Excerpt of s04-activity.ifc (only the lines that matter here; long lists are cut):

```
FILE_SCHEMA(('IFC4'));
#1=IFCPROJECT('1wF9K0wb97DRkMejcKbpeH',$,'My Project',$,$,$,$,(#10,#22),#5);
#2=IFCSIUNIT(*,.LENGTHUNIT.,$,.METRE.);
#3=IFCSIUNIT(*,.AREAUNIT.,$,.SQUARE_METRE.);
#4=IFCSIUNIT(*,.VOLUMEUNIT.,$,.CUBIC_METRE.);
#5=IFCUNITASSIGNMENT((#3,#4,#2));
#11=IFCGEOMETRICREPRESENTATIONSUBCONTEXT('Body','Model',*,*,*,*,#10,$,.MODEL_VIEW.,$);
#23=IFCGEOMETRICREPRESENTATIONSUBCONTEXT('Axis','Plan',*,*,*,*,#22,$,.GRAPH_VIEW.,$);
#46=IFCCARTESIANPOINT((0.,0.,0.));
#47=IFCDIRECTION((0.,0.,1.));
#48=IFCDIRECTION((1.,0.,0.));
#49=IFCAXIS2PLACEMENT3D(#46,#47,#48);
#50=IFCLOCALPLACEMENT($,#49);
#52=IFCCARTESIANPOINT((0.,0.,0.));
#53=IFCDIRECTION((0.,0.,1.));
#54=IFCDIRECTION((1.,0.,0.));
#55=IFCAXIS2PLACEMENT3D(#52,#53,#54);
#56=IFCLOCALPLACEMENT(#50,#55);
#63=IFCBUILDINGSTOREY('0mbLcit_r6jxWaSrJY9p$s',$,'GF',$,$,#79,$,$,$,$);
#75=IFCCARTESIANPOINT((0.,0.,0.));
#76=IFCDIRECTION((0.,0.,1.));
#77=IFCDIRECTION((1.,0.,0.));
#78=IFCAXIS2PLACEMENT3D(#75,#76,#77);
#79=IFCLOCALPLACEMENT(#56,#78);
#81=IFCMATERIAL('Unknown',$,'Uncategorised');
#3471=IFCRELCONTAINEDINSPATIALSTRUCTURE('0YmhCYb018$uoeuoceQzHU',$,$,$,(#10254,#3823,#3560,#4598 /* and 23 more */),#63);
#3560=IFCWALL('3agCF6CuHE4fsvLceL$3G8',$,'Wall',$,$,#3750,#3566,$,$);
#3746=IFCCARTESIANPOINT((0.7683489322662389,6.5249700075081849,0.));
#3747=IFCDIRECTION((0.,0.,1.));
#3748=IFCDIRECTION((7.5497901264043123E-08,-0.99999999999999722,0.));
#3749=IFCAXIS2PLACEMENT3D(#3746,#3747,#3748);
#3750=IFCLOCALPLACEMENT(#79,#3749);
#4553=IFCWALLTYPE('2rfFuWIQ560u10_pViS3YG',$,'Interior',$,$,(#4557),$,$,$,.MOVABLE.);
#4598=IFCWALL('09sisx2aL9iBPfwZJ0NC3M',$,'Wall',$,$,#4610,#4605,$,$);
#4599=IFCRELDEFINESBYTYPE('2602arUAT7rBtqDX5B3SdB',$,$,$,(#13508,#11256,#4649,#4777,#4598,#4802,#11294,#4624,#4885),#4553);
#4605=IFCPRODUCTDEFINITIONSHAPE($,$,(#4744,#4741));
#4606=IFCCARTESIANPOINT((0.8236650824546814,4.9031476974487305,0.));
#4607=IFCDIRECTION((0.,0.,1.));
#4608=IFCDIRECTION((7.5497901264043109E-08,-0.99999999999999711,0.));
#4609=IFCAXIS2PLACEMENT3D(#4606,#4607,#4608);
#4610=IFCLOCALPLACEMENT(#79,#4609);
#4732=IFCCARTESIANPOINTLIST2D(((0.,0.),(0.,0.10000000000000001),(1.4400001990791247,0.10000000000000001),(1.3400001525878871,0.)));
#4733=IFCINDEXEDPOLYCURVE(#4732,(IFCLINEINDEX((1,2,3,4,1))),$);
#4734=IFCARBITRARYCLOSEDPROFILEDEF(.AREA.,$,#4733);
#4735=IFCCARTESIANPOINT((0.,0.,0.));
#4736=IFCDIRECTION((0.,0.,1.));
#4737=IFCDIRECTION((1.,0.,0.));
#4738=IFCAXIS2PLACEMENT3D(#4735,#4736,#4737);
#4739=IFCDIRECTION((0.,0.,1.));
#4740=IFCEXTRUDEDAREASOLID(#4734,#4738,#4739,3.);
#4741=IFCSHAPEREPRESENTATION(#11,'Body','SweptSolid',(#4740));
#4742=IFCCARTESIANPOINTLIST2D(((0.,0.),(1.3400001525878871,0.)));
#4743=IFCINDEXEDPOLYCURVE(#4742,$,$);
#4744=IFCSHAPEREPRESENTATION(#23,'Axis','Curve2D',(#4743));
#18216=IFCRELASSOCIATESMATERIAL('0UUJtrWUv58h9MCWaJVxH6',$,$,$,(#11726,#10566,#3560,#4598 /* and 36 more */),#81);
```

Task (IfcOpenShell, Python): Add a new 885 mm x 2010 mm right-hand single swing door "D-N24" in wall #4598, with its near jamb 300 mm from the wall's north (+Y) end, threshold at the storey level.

```python
import numpy as np
import ifcopenshell
import ifcopenshell.api.feature
import ifcopenshell.api.geometry
import ifcopenshell.api.root
import ifcopenshell.api.spatial
import ifcopenshell.geom
import ifcopenshell.util.element
import ifcopenshell.util.placement
import ifcopenshell.util.representation
import ifcopenshell.util.shape
import ifcopenshell.util.unit

model = ifcopenshell.open("s04-activity.ifc")
unit_scale = ifcopenshell.util.unit.calculate_unit_scale(model)
settings = ifcopenshell.geom.settings()


def volume(element):
    """Net volume in cubic metres, openings subtracted."""
    shape = ifcopenshell.geom.create_shape(settings, element)
    return ifcopenshell.util.shape.get_volume(shape.geometry)


wall = model.by_guid("09sisx2aL9iBPfwZJ0NC3M")
storey = ifcopenshell.util.element.get_container(wall, ifc_class="IfcBuildingStorey")
context = ifcopenshell.util.representation.get_context(model, "Model", "Body", "MODEL_VIEW")
before = volume(wall)

width, height, from_end, sill = 0.885, 2.01, 0.3, 0.0  # metres

# The wall runs along its own X axis, and the end named is its -X end.
wall_shape = ifcopenshell.geom.create_shape(settings, wall)
x, y, z = ifcopenshell.util.shape.get_vertices(wall_shape.geometry).T
start = x.min() + from_end
face, thickness = float(y.min()), float(y.max() - y.min())
wall_matrix = ifcopenshell.util.placement.get_local_placement(wall.ObjectPlacement)
level = ifcopenshell.util.placement.get_local_placement(storey.ObjectPlacement)[2, 3]


def in_wall(x, y):
    """Placement at x, y metres in the wall's axes, at sill height."""
    matrix = wall_matrix.copy()
    matrix[:, 3] = wall_matrix @ np.array([x / unit_scale, y / unit_scale, 0.0, 1.0])
    matrix[2, 3] = level + sill / unit_scale
    return matrix


# Opening: a box that overshoots both wall faces by 50 mm.
opening = ifcopenshell.api.root.create_entity(model, ifc_class="IfcOpeningElement", predefined_type="OPENING")
box = ifcopenshell.api.geometry.add_wall_representation(
    model, context=context, length=width, height=height, thickness=thickness + 0.1
)
ifcopenshell.api.geometry.assign_representation(model, product=opening, representation=box)
ifcopenshell.api.geometry.edit_object_placement(model, product=opening, matrix=in_wall(start, face - 0.05), is_si=False)
ifcopenshell.api.feature.add_feature(model, feature=opening, element=wall)

door = ifcopenshell.api.root.create_entity(model, ifc_class="IfcDoor", name="D-N24", predefined_type="DOOR")
door.OverallWidth, door.OverallHeight = width / unit_scale, height / unit_scale
door.OperationType = "SINGLE_SWING_RIGHT"
body = ifcopenshell.api.geometry.add_door_representation(
    model,
    context=context,
    overall_width=door.OverallWidth,
    overall_height=door.OverallHeight,
    operation_type="SINGLE_SWING_RIGHT",
    lining_properties={"LiningDepth": thickness / unit_scale, "ThresholdDepth": thickness / unit_scale},
)
ifcopenshell.api.geometry.assign_representation(model, product=door, representation=body)
ifcopenshell.api.spatial.assign_container(model, products=[door], relating_structure=storey)
ifcopenshell.api.feature.add_filling(model, opening=opening, element=door)

# The lining spans the wall, so the door starts at the wall face.
ifcopenshell.api.geometry.edit_object_placement(model, product=door, matrix=in_wall(start, face), is_si=False)

after = volume(wall)

print(f"wall volume {before:.3f} -> {after:.3f} m3")

model.write("s04-activity_updated.ifc")
```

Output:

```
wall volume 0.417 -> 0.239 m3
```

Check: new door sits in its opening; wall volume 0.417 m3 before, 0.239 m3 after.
